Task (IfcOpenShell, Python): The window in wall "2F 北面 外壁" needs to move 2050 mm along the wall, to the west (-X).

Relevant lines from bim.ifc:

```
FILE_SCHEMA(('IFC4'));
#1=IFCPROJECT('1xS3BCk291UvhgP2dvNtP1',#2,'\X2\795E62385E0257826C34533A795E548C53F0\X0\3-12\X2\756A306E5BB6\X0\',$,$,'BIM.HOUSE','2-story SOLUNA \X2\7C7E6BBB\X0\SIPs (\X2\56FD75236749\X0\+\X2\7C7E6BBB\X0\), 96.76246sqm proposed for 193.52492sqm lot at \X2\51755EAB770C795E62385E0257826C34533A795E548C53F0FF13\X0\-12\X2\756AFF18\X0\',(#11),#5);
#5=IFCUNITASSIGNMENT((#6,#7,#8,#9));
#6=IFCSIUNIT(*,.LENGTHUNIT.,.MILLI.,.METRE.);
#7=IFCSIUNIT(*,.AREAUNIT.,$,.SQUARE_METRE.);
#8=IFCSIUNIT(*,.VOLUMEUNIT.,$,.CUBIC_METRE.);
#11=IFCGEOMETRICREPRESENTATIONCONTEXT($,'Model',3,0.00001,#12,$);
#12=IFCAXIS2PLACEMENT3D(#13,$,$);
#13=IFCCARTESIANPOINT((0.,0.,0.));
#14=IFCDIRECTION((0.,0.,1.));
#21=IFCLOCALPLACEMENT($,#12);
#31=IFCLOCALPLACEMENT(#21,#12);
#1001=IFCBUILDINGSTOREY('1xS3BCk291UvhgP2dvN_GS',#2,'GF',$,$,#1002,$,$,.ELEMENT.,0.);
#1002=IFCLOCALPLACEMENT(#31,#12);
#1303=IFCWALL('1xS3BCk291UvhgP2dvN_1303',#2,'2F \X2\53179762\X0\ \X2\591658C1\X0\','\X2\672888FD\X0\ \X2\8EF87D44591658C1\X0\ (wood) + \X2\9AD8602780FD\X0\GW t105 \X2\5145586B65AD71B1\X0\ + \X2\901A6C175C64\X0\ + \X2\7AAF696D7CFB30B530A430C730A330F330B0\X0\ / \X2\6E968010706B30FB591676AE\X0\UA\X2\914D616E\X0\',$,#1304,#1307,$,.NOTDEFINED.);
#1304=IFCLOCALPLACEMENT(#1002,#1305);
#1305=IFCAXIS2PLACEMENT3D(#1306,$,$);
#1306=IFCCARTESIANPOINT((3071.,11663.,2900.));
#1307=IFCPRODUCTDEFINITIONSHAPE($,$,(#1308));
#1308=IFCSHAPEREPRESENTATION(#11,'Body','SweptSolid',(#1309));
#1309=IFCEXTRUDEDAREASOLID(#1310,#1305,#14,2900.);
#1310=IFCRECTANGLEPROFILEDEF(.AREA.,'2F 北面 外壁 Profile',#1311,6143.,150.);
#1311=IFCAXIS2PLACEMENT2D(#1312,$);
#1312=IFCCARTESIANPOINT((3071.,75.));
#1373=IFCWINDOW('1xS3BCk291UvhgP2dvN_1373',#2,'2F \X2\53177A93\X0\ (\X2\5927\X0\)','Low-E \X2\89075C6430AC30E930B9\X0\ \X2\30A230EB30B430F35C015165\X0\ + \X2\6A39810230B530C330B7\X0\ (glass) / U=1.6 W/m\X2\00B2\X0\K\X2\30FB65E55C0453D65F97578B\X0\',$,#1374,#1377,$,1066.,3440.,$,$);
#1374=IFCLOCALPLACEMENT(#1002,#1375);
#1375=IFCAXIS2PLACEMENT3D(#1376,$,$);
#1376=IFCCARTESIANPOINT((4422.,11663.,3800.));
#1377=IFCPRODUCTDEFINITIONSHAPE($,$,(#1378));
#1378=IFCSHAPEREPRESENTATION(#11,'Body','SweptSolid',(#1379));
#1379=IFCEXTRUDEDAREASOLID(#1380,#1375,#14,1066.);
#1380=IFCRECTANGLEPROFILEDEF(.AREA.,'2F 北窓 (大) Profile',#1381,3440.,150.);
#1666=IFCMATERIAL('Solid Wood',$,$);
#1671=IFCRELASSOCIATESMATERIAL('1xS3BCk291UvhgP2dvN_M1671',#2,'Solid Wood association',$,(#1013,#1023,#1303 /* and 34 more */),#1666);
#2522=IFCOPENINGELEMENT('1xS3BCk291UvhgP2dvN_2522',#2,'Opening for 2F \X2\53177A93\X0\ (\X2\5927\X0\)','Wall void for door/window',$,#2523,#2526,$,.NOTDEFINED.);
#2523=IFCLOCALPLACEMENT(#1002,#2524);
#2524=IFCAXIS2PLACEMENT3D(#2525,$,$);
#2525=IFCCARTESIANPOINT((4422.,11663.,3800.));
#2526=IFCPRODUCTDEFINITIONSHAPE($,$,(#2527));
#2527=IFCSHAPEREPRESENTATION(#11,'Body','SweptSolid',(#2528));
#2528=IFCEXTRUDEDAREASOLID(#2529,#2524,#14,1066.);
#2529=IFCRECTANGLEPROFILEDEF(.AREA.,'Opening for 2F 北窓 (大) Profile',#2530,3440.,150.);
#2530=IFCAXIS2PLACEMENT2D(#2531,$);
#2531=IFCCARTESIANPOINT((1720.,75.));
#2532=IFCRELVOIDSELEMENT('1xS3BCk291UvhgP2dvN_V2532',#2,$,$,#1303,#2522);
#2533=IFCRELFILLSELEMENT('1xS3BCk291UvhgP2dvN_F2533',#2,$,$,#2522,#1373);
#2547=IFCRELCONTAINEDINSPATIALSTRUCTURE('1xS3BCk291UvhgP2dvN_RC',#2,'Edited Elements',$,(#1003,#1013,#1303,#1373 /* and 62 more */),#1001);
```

```python
import ifcopenshell
import ifcopenshell.api.geometry
import ifcopenshell.util.placement
import ifcopenshell.util.unit

model = ifcopenshell.open("bim.ifc")
unit_scale = ifcopenshell.util.unit.calculate_unit_scale(model)

window = model.by_guid("1xS3BCk291UvhgP2dvN_1373")
opening = window.FillsVoids[0].RelatingOpeningElement
wall = opening.VoidsElements[0].RelatingBuildingElement

wall_matrix = ifcopenshell.util.placement.get_local_placement(wall.ObjectPlacement)
shift = wall_matrix[:3, 0] * -2.05 / unit_scale
before = ifcopenshell.util.placement.get_local_placement(window.ObjectPlacement)[:3, 3].copy()

# The window is not placed relative to its opening, so move both.
for product in (opening, window):
    matrix = ifcopenshell.util.placement.get_local_placement(product.ObjectPlacement)
    matrix[:3, 3] += shift
    ifcopenshell.api.geometry.edit_object_placement(model, product=product, matrix=matrix, is_si=False)

after = ifcopenshell.util.placement.get_local_placement(window.ObjectPlacement)[:3, 3]
print("window moved by", (after - before).round(3) + 0.0)

model.write("bim-out.ifc")
```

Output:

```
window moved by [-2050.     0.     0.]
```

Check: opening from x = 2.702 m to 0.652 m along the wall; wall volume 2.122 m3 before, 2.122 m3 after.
